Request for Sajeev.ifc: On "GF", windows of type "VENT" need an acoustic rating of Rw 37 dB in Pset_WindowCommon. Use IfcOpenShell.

First a look at what the model holds.

```python
import ifcopenshell
import ifcopenshell.util.element

model = ifcopenshell.open("Sajeev.ifc")
print(model.schema)
storey = next(s for s in model.by_type("IfcBuildingStorey") if s.Name == "GF")
windows = [e for e in ifcopenshell.util.element.get_decomposition(storey) if e.is_a("IfcWindow")]
seen = {}
for e in windows:
    element_type = ifcopenshell.util.element.get_type(e)
    key = (element_type.Name if element_type != e and element_type else None, ifcopenshell.util.element.get_pset(e, "Pset_WindowCommon", "AcousticRating"))
    seen[key] = seen.get(key, 0) + 1
for (name, value), count in sorted(seen.items(), key=str):
    print(count, "x", name, "|", value)
```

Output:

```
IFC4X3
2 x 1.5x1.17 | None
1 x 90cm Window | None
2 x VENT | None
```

```python
import ifcopenshell
import ifcopenshell.api.pset
import ifcopenshell.util.element

model = ifcopenshell.open("Sajeev.ifc")

storey = next(s for s in model.by_type("IfcBuildingStorey") if s.Name == "GF")
windows = [e for e in ifcopenshell.util.element.get_decomposition(storey) if e.is_a("IfcWindow")]

count = 0
for e in windows:
    element_type = ifcopenshell.util.element.get_type(e)
    if element_type in (None, e) or element_type.Name != "VENT":
        continue
    # add_pset returns the element's existing set when there is one.
    pset = ifcopenshell.api.pset.add_pset(model, product=e, name="Pset_WindowCommon")
    ifcopenshell.api.pset.edit_pset(model, pset=pset, properties={"AcousticRating": "Rw 37 dB"})
    count += 1

print(count, "windows updated")

model.write("Sajeev_edited.ifc")
```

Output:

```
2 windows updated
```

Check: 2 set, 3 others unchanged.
